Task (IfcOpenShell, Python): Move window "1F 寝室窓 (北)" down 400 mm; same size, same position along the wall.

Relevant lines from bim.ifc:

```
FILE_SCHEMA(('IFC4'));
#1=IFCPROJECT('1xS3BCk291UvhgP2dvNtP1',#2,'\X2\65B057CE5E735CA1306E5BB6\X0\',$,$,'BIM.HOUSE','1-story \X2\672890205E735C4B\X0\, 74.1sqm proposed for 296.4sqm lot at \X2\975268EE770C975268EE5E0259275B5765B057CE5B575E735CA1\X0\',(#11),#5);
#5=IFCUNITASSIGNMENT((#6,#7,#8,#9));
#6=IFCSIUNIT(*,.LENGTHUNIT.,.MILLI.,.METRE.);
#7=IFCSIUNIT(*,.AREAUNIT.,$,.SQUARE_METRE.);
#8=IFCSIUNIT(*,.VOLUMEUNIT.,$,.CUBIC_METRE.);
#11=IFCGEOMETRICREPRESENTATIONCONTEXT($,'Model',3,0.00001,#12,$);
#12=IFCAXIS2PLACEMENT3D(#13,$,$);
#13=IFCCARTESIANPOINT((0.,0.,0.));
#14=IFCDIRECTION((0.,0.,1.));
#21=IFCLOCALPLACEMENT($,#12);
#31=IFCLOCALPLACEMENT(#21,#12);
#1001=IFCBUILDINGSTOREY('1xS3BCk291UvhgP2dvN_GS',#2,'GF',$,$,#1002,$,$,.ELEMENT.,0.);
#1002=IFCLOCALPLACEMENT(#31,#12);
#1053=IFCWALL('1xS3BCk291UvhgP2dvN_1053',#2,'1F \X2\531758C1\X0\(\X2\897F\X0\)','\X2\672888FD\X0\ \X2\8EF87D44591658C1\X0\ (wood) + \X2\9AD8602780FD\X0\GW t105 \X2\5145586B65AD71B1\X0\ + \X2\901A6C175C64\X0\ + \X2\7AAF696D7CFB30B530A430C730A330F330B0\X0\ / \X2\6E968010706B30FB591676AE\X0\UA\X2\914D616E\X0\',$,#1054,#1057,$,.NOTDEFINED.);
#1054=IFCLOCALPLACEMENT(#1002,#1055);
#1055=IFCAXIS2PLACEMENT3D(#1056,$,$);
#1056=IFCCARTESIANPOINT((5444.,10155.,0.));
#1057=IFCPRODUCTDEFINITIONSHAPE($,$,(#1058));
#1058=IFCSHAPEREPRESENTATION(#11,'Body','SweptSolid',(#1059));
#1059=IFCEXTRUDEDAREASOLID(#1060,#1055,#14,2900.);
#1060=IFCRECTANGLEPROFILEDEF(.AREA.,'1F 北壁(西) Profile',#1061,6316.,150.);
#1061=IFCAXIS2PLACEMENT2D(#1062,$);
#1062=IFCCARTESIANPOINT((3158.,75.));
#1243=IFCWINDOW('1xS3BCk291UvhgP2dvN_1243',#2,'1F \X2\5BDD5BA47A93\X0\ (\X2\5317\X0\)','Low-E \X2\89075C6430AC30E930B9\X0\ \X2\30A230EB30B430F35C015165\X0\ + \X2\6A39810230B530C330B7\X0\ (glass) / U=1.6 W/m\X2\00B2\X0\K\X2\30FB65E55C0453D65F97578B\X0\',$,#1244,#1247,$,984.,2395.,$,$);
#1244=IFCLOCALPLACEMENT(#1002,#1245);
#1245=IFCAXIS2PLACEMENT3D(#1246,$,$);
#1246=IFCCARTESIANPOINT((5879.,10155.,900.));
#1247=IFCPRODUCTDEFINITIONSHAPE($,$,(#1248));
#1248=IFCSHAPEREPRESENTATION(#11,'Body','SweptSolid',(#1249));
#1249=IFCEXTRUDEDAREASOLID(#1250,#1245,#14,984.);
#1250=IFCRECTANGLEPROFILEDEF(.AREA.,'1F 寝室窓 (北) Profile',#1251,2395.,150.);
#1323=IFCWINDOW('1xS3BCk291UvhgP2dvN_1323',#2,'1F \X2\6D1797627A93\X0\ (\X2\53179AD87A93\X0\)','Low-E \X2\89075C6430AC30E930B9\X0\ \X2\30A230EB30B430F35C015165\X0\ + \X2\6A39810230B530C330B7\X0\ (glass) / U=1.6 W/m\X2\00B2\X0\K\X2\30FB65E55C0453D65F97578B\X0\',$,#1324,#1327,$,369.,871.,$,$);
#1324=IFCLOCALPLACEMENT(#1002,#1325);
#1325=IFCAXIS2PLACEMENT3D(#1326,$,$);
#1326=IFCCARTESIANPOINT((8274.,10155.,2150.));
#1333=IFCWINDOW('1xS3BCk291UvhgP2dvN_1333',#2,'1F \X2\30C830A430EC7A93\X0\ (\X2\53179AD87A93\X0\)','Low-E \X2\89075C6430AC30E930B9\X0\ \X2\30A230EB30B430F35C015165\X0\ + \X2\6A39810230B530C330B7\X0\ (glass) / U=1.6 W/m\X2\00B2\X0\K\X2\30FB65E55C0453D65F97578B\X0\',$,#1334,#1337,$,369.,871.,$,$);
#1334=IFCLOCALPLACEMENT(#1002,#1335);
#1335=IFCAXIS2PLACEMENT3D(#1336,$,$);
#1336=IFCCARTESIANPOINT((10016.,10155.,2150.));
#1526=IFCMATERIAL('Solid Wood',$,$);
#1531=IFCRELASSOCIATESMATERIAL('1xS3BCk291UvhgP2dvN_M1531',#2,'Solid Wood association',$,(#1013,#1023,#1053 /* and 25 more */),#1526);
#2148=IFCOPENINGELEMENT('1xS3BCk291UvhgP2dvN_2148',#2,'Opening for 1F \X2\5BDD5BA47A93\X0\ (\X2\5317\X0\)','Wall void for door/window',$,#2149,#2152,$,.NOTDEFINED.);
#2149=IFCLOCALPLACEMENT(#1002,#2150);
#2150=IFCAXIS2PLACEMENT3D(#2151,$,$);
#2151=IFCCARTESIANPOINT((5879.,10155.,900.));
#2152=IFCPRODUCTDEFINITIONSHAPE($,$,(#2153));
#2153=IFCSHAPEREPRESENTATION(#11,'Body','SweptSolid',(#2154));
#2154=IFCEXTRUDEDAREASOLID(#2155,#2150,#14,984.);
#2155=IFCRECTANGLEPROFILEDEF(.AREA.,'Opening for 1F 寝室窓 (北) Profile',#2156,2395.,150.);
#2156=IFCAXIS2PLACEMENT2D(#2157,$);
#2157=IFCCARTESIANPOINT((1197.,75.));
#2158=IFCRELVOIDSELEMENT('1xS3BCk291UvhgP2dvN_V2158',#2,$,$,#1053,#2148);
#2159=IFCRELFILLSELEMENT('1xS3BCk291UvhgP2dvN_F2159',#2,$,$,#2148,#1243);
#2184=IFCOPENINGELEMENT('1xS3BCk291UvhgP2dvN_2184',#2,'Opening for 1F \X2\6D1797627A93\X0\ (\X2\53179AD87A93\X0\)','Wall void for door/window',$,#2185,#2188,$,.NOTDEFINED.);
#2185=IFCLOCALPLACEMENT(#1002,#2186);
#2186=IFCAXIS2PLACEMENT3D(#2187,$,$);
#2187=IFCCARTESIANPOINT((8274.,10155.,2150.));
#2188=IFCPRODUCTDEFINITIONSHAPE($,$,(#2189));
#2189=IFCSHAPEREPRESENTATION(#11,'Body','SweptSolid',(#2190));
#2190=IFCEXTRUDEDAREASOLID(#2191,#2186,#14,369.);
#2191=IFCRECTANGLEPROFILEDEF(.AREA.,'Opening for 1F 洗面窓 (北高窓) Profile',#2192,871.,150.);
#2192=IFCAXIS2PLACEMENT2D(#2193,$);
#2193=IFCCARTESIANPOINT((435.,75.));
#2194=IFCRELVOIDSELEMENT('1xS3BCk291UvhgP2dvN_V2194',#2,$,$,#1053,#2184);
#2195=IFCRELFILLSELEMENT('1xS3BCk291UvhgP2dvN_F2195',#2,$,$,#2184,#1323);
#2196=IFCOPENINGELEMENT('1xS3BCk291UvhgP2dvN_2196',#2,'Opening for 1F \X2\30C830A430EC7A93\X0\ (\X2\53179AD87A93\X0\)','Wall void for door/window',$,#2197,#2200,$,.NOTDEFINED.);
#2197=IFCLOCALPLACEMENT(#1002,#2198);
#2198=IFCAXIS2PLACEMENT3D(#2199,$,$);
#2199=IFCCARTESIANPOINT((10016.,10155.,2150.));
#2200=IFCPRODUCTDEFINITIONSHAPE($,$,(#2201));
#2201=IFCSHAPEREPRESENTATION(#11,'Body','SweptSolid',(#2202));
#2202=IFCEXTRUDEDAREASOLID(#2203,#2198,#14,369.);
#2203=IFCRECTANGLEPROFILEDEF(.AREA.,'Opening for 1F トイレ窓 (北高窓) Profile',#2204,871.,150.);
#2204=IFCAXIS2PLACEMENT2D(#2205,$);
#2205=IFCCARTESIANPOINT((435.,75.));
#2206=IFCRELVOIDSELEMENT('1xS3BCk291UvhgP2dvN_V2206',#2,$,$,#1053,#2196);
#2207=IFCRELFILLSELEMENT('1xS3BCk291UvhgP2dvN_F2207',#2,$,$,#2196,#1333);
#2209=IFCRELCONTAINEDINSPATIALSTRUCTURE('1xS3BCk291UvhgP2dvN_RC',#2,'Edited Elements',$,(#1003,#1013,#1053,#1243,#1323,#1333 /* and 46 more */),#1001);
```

```python
import numpy as np
import ifcopenshell
import ifcopenshell.api.geometry
import ifcopenshell.util.placement
import ifcopenshell.util.unit

model = ifcopenshell.open("bim.ifc")
unit_scale = ifcopenshell.util.unit.calculate_unit_scale(model)

window = model.by_guid("1xS3BCk291UvhgP2dvN_1243")
opening = window.FillsVoids[0].RelatingOpeningElement
dz = -400.0

shift = np.array([0.0, 0.0, dz])
# The window is not placed relative to its opening, so move both.
for product in (opening, window):
    matrix = ifcopenshell.util.placement.get_local_placement(product.ObjectPlacement)
    matrix[:3, 3] += shift
    ifcopenshell.api.geometry.edit_object_placement(model, product=product, matrix=matrix, is_si=False)

print(f"moved by {dz * unit_scale:+.3f} m")

model.write("bim_edited.ifc")
```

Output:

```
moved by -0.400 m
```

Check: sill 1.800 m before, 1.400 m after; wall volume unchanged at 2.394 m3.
